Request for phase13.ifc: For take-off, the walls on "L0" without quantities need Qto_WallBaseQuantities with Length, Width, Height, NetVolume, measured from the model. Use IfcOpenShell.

First a look at what the model holds.

```python
import ifcopenshell
import ifcopenshell.util.element
import ifcopenshell.util.unit

model = ifcopenshell.open("phase13.ifc")
print(model.schema)
for unit_type in ("LENGTHUNIT", "AREAUNIT", "VOLUMEUNIT"):
    print(unit_type, ifcopenshell.util.unit.calculate_unit_scale(model, unit_type))
storey = next(s for s in model.by_type("IfcBuildingStorey") if s.Name == "L0")
walls = [e for e in ifcopenshell.util.element.get_decomposition(storey) if e.is_a("IfcWall")]
for e in sorted(walls, key=lambda e: e.id()):
    print(e.id(), e.is_a(), e.Name, list(ifcopenshell.util.element.get_psets(e, qtos_only=True)), sep=" | ")
```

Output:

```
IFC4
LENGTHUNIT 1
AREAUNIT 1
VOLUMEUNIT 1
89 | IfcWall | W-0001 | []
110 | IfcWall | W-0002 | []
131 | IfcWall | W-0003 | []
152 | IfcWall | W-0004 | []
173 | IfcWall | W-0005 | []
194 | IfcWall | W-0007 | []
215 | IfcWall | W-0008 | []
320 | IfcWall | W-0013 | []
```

```python
import ifcopenshell
import ifcopenshell.api.pset
import ifcopenshell.geom
import ifcopenshell.util.element
import ifcopenshell.util.shape
import ifcopenshell.util.unit

model = ifcopenshell.open("phase13.ifc")
unit_scale = ifcopenshell.util.unit.calculate_unit_scale(model)
volume_scale = ifcopenshell.util.unit.calculate_unit_scale(model, "VOLUMEUNIT")
settings = ifcopenshell.geom.settings()

storey = next(s for s in model.by_type("IfcBuildingStorey") if s.Name == "L0")
walls = [e for e in ifcopenshell.util.element.get_decomposition(storey) if e.is_a("IfcWall")]

for e in sorted(walls, key=lambda e: e.id()):
    if ifcopenshell.util.element.get_psets(e, qtos_only=True, should_inherit=False):
        continue
    # Geometry comes back in metres, in the element's own axes.
    shape = ifcopenshell.geom.create_shape(settings, e)
    values = {
        "Length": ifcopenshell.util.shape.get_x(shape.geometry) / unit_scale,
        "Width": ifcopenshell.util.shape.get_y(shape.geometry) / unit_scale,
        "Height": ifcopenshell.util.shape.get_z(shape.geometry) / unit_scale,
        "NetVolume": ifcopenshell.util.shape.get_volume(shape.geometry) / volume_scale,
    }
    qto = ifcopenshell.api.pset.add_qto(model, product=e, name="Qto_WallBaseQuantities")
    ifcopenshell.api.pset.edit_qto(model, qto=qto, properties=values)
    print(e.id(), {k: round(v, 3) for k, v in values.items()})

model.write("phase13-out.ifc")
```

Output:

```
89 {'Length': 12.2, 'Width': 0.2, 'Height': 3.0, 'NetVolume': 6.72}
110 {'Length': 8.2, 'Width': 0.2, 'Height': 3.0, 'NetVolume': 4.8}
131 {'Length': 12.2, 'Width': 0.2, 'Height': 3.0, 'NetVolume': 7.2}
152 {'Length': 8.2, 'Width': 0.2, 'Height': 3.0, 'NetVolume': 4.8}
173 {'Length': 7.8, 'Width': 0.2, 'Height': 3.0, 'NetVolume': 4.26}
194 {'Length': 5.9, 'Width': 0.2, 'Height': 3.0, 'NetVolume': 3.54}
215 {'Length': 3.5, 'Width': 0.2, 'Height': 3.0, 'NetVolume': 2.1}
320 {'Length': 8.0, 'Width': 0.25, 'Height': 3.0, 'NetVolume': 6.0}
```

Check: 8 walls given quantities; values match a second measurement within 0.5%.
